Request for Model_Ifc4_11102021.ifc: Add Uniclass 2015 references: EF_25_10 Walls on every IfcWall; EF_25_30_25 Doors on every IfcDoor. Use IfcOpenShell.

First a look at what the model holds.

```python
import ifcopenshell

model = ifcopenshell.open("Model_Ifc4_11102021.ifc")
print(model.schema)
print("classifications:", [c.Name for c in model.by_type("IfcClassification")])
for ifc_class in ("IfcDoor", "IfcRoof", "IfcStair", "IfcWall", "IfcWindow"):
    print(ifc_class, len(model.by_type(ifc_class)))
```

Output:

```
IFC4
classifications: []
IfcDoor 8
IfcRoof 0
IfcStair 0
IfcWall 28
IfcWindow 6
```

```python
import ifcopenshell
import ifcopenshell.api.classification

model = ifcopenshell.open("Model_Ifc4_11102021.ifc")

system = ifcopenshell.api.classification.add_classification(model, classification="Uniclass 2015")

codes = {
    "IfcWall": ("EF_25_10", "Walls"),
    "IfcDoor": ("EF_25_30_25", "Doors"),
}
for ifc_class, (code, name) in codes.items():
    products = model.by_type(ifc_class)
    ifcopenshell.api.classification.add_reference(
        model, products=products, classification=system, identification=code, name=name
    )
    print(code, len(products))

model.write("Model_Ifc4_11102021_rev.ifc")
```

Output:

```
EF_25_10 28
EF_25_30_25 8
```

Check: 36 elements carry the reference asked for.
